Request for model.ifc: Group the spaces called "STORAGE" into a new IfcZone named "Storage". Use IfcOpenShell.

First a look at what the model holds.

```python
import ifcopenshell

model = ifcopenshell.open("model.ifc")
print(model.schema)
seen = {}
for space in model.by_type("IfcSpace"):
    seen[space.LongName] = seen.get(space.LongName, 0) + 1
for name, count in sorted(seen.items(), key=str):
    print(count, "x", name)
print("zones:", [z.Name for z in model.by_type("IfcZone")][:20])
```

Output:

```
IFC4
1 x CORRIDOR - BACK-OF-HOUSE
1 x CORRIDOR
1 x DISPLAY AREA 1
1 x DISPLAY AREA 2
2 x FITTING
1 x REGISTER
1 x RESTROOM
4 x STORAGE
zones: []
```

```python
import ifcopenshell
import ifcopenshell.api.group
import ifcopenshell.api.root

model = ifcopenshell.open("model.ifc")

names = {"STORAGE"}
spaces = [s for s in model.by_type("IfcSpace") if s.LongName in names]

zone = ifcopenshell.api.root.create_entity(model, ifc_class="IfcZone", name="Storage")
ifcopenshell.api.group.assign_group(model, products=spaces, group=zone)
print(len(spaces), "spaces in", zone.Name)

model.write("model_rev.ifc")
```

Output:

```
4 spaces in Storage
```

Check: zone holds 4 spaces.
